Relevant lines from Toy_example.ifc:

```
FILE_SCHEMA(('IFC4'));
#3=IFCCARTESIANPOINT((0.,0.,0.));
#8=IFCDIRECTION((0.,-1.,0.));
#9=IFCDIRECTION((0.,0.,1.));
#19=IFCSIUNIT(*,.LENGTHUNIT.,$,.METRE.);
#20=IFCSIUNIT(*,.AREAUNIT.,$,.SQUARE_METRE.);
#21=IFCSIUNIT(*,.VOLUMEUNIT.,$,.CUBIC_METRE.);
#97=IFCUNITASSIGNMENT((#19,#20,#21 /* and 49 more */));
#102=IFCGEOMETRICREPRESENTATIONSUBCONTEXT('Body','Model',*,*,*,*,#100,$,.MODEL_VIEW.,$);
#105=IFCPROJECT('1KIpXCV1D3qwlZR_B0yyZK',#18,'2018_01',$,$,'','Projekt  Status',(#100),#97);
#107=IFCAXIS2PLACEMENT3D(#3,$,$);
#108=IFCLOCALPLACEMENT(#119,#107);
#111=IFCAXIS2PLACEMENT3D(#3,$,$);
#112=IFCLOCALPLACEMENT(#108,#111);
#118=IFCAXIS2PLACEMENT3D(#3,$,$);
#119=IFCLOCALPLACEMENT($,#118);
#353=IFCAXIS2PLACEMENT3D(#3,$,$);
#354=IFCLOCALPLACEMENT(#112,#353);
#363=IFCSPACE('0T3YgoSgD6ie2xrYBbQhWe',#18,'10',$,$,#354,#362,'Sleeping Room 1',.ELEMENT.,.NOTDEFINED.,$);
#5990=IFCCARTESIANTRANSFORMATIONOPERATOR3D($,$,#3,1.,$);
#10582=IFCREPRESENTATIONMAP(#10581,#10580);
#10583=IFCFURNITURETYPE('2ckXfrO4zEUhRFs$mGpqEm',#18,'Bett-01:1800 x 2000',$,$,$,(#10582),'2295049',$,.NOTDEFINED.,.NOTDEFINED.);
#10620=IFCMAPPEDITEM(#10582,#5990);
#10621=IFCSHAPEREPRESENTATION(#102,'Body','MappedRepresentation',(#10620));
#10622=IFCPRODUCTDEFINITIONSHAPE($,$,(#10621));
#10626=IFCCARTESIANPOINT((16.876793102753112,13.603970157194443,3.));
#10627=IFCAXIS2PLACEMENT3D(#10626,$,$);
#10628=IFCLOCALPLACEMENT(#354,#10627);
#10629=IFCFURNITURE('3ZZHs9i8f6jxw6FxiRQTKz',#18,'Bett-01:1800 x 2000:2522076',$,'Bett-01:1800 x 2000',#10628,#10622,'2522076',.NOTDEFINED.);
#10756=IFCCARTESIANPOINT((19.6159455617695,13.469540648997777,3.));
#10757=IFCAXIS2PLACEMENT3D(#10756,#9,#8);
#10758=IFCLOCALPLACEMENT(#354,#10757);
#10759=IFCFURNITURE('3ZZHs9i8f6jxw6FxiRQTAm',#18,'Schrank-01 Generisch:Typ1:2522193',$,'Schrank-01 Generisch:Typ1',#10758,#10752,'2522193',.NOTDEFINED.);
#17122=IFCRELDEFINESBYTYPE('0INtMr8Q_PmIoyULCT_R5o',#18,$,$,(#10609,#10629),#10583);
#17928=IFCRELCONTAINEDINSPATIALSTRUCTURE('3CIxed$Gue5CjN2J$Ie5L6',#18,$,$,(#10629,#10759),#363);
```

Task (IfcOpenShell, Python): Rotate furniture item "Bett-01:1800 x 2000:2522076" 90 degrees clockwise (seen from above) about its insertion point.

```python
import ifcopenshell
import ifcopenshell.api.geometry
import ifcopenshell.util.placement

model = ifcopenshell.open("Toy_example.ifc")

item = model.by_id(10629)
matrix = ifcopenshell.util.placement.get_local_placement(item.ObjectPlacement)
matrix = matrix @ ifcopenshell.util.placement.rotation(-90, "Z")
ifcopenshell.api.geometry.edit_object_placement(model, product=item, matrix=matrix, is_si=False)

print(ifcopenshell.util.placement.get_local_placement(item.ObjectPlacement).round(3) + 0.0)

model.write("Toy_example_rev.ifc")
```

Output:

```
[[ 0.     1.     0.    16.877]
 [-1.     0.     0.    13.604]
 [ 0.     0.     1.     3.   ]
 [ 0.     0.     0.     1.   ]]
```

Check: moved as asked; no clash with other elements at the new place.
